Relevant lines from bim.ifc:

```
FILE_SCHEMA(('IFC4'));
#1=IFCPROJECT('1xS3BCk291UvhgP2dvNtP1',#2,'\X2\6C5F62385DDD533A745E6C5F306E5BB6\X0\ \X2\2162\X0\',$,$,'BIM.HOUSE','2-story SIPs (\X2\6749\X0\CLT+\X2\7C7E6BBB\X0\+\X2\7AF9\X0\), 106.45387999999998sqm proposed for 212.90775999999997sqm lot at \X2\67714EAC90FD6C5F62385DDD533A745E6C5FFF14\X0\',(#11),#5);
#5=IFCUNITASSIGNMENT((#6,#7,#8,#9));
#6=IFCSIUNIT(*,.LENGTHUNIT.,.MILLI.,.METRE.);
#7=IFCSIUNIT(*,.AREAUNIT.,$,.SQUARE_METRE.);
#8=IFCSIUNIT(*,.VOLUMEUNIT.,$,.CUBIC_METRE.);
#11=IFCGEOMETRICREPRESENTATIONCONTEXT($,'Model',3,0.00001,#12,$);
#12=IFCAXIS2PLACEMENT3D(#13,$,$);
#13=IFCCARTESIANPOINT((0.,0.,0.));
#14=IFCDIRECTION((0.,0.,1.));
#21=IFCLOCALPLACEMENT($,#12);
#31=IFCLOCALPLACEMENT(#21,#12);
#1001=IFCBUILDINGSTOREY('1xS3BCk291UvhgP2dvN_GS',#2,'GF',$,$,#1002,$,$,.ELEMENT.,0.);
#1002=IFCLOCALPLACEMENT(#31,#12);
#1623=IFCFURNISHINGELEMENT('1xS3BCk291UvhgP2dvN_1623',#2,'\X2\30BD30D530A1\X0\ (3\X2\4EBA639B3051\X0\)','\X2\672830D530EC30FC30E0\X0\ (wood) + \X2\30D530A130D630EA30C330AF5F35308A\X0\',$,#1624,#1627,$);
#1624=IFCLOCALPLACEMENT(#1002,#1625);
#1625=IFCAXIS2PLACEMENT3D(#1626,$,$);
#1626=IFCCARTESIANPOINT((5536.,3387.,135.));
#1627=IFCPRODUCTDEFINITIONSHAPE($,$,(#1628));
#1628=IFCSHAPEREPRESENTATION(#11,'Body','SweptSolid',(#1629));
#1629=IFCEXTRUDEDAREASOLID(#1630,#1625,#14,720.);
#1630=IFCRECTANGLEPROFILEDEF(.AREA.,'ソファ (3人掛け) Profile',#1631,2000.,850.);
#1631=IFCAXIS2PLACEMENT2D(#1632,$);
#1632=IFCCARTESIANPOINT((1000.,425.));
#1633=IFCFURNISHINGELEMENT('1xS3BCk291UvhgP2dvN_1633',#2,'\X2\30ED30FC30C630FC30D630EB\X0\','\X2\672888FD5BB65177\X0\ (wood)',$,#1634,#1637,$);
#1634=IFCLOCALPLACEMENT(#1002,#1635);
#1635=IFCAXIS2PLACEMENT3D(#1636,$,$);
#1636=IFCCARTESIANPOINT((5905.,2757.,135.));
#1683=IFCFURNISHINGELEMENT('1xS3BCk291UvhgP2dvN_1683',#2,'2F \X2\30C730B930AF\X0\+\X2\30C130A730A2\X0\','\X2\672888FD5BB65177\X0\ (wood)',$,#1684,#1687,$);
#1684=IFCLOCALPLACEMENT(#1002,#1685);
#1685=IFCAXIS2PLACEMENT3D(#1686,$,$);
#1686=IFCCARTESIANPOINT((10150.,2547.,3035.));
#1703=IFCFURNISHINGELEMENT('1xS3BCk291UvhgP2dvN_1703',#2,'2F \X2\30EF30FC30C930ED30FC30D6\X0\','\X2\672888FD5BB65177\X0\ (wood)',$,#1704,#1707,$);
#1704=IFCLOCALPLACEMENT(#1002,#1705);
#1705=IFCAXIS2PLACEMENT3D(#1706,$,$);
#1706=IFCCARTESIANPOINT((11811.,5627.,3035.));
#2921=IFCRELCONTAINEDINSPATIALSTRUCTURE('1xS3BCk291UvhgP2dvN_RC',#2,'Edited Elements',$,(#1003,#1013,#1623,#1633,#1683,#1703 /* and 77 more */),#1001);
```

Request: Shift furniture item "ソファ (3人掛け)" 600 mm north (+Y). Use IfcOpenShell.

```python
import ifcopenshell
import ifcopenshell.api.geometry
import ifcopenshell.util.placement

model = ifcopenshell.open("bim.ifc")

item = model.by_guid("1xS3BCk291UvhgP2dvN_1623")
matrix = ifcopenshell.util.placement.get_local_placement(item.ObjectPlacement)
matrix[1, 3] += 600.0
ifcopenshell.api.geometry.edit_object_placement(model, product=item, matrix=matrix, is_si=False)

print(ifcopenshell.util.placement.get_local_placement(item.ObjectPlacement).round(3) + 0.0)

model.write("bim_v2.ifc")
```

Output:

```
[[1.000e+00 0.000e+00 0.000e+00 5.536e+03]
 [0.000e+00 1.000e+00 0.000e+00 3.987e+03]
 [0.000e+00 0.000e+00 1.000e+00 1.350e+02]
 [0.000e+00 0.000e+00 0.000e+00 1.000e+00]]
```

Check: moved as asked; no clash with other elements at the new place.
